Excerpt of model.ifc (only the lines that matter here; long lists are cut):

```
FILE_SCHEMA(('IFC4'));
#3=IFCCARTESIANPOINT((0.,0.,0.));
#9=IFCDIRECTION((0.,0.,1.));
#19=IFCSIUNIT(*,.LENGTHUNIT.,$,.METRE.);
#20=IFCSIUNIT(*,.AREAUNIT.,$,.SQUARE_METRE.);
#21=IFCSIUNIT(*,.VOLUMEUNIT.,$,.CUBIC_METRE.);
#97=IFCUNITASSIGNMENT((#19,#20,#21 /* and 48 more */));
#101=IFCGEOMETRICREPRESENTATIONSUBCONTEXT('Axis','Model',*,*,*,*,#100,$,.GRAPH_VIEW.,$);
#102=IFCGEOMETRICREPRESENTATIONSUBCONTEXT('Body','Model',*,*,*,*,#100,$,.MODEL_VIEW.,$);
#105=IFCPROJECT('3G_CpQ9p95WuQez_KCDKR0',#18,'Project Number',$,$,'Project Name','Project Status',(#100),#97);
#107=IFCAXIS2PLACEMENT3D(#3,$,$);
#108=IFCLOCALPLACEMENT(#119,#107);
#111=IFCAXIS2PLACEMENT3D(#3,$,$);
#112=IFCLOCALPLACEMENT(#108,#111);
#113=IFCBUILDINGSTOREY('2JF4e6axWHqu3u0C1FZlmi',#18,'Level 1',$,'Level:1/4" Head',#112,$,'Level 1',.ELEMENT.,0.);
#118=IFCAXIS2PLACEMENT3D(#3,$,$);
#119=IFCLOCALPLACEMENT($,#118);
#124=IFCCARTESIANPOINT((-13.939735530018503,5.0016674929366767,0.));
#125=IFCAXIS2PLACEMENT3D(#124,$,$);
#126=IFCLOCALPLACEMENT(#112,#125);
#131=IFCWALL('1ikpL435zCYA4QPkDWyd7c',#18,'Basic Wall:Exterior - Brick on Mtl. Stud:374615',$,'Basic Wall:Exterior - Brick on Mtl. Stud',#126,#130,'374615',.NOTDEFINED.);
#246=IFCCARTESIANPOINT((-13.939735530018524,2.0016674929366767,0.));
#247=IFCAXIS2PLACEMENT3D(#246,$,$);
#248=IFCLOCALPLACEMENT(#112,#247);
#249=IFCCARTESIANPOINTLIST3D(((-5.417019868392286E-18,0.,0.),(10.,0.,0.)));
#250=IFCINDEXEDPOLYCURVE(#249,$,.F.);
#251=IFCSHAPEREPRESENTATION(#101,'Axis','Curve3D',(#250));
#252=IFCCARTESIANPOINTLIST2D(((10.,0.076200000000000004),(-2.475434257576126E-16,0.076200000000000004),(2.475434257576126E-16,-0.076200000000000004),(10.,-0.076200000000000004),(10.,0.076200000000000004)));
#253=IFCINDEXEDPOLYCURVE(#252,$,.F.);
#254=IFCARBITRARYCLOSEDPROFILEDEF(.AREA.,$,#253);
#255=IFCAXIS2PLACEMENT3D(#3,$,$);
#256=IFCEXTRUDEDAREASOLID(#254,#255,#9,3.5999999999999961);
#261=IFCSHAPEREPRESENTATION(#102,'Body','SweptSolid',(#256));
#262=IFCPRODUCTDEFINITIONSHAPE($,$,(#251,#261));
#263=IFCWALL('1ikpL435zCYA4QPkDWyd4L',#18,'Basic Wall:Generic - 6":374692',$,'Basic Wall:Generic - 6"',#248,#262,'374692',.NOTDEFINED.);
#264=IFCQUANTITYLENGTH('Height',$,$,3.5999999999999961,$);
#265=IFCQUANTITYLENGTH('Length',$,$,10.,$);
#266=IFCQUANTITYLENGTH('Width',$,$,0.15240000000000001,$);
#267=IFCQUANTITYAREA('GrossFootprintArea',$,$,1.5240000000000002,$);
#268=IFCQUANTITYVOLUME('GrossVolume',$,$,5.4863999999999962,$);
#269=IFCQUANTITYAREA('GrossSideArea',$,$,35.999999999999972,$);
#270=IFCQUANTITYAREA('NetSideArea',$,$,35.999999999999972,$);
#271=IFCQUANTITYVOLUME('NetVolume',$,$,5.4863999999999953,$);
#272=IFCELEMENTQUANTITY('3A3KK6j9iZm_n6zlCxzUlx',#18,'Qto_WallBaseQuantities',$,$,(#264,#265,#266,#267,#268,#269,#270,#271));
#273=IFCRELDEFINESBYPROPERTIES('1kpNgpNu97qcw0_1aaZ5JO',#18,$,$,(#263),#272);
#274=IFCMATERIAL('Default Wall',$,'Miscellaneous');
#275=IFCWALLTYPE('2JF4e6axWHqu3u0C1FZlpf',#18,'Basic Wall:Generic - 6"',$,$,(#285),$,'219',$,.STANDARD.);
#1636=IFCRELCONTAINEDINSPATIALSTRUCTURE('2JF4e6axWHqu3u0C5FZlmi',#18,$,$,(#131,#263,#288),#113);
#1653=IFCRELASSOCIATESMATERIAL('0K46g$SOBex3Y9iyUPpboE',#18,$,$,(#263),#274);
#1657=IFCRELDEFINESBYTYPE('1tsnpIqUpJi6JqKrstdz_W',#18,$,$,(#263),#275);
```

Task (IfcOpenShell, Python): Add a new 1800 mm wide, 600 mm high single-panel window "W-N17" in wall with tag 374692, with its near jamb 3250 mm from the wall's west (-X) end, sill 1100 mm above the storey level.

```python
import numpy as np
import ifcopenshell
import ifcopenshell.api.feature
import ifcopenshell.api.geometry
import ifcopenshell.api.pset
import ifcopenshell.api.root
import ifcopenshell.api.spatial
import ifcopenshell.geom
import ifcopenshell.util.element
import ifcopenshell.util.placement
import ifcopenshell.util.representation
import ifcopenshell.util.shape
import ifcopenshell.util.unit

model = ifcopenshell.open("model.ifc")
unit_scale = ifcopenshell.util.unit.calculate_unit_scale(model)
area_scale = ifcopenshell.util.unit.calculate_unit_scale(model, "AREAUNIT")
volume_scale = ifcopenshell.util.unit.calculate_unit_scale(model, "VOLUMEUNIT")
settings = ifcopenshell.geom.settings()


def volume(element):
    """Net volume in cubic metres, openings subtracted."""
    shape = ifcopenshell.geom.create_shape(settings, element)
    return ifcopenshell.util.shape.get_volume(shape.geometry)


wall = model.by_id(263)
storey = ifcopenshell.util.element.get_container(wall, ifc_class="IfcBuildingStorey")
context = ifcopenshell.util.representation.get_context(model, "Model", "Body", "MODEL_VIEW")
before = volume(wall)

width, height, from_end, sill = 1.8, 0.6, 3.25, 1.1  # metres

# The wall runs along its own X axis, and the end named is its -X end.
wall_shape = ifcopenshell.geom.create_shape(settings, wall)
x, y, z = ifcopenshell.util.shape.get_vertices(wall_shape.geometry).T
start = x.min() + from_end
face, thickness = float(y.min()), float(y.max() - y.min())
wall_matrix = ifcopenshell.util.placement.get_local_placement(wall.ObjectPlacement)
level = ifcopenshell.util.placement.get_local_placement(storey.ObjectPlacement)[2, 3]


def in_wall(x, y):
    """Placement at x, y metres in the wall's axes, at sill height."""
    matrix = wall_matrix.copy()
    matrix[:, 3] = wall_matrix @ np.array([x / unit_scale, y / unit_scale, 0.0, 1.0])
    matrix[2, 3] = level + sill / unit_scale
    return matrix


# Opening: a box that overshoots both wall faces by 50 mm.
opening = ifcopenshell.api.root.create_entity(model, ifc_class="IfcOpeningElement", predefined_type="OPENING")
box = ifcopenshell.api.geometry.add_wall_representation(
    model, context=context, length=width, height=height, thickness=thickness + 0.1
)
ifcopenshell.api.geometry.assign_representation(model, product=opening, representation=box)
ifcopenshell.api.geometry.edit_object_placement(model, product=opening, matrix=in_wall(start, face - 0.05), is_si=False)
ifcopenshell.api.feature.add_feature(model, feature=opening, element=wall)

window = ifcopenshell.api.root.create_entity(model, ifc_class="IfcWindow", name="W-N17", predefined_type="WINDOW")
window.OverallWidth, window.OverallHeight = width / unit_scale, height / unit_scale
window.PartitioningType = "SINGLE_PANEL"
body = ifcopenshell.api.geometry.add_window_representation(
    model,
    context=context,
    overall_width=window.OverallWidth,
    overall_height=window.OverallHeight,
    partition_type="SINGLE_PANEL",
)
ifcopenshell.api.geometry.assign_representation(model, product=window, representation=body)
ifcopenshell.api.spatial.assign_container(model, products=[window], relating_structure=storey)
ifcopenshell.api.feature.add_filling(model, opening=opening, element=window)

# Centre the window in the wall's thickness.
ifcopenshell.api.geometry.edit_object_placement(model, product=window, matrix=in_wall(start, face), is_si=False)
window_shape = ifcopenshell.geom.create_shape(settings, window)
depth = ifcopenshell.util.shape.get_vertices(window_shape.geometry)[:, 1]
offset = face + thickness / 2 - (depth.min() + depth.max()) / 2
ifcopenshell.api.geometry.edit_object_placement(model, product=window, matrix=in_wall(start, offset), is_si=False)

after = volume(wall)

# Update the wall's stored quantities.
qto = model.by_id(ifcopenshell.util.element.get_pset(wall, "Qto_WallBaseQuantities", should_inherit=False)["id"])
ifcopenshell.api.pset.edit_qto(model, qto=qto, properties={
    "NetSideArea": after / thickness / area_scale,
    "NetVolume": after / volume_scale,
})

print(f"wall volume {before:.3f} -> {after:.3f} m3")

model.write("model_edited.ifc")
```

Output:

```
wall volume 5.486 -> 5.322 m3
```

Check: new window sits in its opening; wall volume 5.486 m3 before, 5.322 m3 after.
